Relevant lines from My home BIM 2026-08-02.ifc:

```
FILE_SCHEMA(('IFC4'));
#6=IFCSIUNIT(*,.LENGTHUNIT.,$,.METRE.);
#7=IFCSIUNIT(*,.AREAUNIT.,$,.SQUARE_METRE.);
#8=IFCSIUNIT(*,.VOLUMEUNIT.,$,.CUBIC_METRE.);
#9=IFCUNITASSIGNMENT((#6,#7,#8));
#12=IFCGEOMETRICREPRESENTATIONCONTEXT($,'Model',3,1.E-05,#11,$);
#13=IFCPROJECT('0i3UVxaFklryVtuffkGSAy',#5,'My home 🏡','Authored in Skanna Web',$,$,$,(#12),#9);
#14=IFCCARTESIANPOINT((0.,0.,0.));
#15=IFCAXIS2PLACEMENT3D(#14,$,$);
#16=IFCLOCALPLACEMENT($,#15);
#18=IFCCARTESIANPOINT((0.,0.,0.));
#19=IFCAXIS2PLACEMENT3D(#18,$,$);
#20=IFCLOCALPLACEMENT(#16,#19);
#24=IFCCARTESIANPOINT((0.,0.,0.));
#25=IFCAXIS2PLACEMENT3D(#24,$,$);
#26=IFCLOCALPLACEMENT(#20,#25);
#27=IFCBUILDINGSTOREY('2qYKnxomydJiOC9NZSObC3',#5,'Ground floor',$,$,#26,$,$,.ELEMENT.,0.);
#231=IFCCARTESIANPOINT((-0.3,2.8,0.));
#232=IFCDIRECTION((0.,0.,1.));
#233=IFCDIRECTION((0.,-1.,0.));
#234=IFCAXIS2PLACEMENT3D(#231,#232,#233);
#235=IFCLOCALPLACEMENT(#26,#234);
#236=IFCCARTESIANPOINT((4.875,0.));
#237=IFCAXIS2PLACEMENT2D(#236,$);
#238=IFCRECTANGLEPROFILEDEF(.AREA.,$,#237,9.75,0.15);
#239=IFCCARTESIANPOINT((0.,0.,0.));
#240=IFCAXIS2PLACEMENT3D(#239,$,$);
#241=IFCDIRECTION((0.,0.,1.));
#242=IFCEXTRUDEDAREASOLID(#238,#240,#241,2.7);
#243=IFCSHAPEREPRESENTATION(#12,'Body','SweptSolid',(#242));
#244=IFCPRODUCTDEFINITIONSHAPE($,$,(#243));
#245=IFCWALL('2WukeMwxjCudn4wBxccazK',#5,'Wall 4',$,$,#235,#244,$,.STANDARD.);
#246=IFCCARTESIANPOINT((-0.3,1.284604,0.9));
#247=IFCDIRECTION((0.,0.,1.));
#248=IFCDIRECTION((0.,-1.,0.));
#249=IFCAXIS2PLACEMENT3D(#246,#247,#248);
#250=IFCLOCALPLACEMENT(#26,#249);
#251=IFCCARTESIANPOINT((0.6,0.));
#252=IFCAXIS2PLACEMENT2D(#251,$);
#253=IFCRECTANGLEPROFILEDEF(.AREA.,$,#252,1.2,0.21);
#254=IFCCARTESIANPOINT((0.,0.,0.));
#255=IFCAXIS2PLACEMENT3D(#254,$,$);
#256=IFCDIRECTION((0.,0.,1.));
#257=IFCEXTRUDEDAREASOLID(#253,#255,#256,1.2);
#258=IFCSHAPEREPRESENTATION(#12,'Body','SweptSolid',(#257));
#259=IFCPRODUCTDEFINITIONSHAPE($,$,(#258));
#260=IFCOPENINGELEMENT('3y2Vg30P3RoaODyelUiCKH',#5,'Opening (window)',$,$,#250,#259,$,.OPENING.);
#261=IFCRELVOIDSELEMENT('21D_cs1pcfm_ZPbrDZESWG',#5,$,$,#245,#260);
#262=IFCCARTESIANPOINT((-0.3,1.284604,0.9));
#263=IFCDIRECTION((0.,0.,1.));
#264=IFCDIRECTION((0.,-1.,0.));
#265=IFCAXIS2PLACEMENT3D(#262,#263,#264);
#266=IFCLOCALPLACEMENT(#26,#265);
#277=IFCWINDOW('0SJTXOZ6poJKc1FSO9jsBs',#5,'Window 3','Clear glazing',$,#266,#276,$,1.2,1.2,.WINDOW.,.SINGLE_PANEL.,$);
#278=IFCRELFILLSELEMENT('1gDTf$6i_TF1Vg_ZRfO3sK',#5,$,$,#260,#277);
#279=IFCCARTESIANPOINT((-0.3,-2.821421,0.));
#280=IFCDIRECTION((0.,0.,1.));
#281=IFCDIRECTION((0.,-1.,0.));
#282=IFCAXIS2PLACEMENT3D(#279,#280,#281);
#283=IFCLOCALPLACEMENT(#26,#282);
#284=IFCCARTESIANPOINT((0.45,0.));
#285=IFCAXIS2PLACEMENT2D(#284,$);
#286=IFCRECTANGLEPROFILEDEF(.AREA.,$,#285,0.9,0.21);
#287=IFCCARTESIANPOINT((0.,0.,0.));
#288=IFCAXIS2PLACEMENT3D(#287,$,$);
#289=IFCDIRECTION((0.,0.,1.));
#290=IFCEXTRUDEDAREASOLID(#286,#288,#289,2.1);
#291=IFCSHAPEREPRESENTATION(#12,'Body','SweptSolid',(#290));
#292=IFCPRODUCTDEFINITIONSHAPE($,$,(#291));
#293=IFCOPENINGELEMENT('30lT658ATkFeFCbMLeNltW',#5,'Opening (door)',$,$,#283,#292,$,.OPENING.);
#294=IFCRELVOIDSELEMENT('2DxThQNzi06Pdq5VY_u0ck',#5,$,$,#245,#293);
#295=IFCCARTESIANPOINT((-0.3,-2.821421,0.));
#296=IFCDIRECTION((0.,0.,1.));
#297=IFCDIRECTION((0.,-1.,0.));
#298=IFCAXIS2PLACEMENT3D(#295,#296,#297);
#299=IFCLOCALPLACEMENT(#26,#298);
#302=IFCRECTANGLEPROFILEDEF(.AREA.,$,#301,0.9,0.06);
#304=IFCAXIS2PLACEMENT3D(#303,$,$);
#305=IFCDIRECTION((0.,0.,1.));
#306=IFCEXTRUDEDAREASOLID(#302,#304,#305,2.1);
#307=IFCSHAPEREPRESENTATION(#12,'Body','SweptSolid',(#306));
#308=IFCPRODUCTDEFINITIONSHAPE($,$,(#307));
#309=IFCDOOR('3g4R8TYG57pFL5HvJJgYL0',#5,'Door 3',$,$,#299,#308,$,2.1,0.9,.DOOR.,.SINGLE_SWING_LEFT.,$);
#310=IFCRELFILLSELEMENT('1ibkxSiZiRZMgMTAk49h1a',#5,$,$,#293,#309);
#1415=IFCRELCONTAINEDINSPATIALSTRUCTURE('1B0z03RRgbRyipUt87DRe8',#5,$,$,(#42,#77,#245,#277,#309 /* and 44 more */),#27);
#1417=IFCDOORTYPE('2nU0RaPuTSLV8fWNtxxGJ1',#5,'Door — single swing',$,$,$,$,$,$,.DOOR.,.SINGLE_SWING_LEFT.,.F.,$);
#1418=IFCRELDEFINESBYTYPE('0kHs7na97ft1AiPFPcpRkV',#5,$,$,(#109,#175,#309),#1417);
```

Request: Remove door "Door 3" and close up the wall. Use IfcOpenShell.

```python
import ifcopenshell
import ifcopenshell.api.feature
import ifcopenshell.api.root
import ifcopenshell.geom
import ifcopenshell.util.shape

model = ifcopenshell.open("My home BIM 2026-08-02.ifc")
settings = ifcopenshell.geom.settings()


def volume(element):
    """Net volume in cubic metres, openings subtracted."""
    shape = ifcopenshell.geom.create_shape(settings, element)
    return ifcopenshell.util.shape.get_volume(shape.geometry)


door = model.by_guid("3g4R8TYG57pFL5HvJJgYL0")
opening = door.FillsVoids[0].RelatingOpeningElement
wall = opening.VoidsElements[0].RelatingBuildingElement
before = volume(wall)

ifcopenshell.api.root.remove_product(model, product=door)
ifcopenshell.api.feature.remove_feature(model, feature=opening)

after = volume(wall)

print(f"wall volume {before:.3f} -> {after:.3f} m3")

model.write("My home BIM 2026-08-02_rev.ifc")
```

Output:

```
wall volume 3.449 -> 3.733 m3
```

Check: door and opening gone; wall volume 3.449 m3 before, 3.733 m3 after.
